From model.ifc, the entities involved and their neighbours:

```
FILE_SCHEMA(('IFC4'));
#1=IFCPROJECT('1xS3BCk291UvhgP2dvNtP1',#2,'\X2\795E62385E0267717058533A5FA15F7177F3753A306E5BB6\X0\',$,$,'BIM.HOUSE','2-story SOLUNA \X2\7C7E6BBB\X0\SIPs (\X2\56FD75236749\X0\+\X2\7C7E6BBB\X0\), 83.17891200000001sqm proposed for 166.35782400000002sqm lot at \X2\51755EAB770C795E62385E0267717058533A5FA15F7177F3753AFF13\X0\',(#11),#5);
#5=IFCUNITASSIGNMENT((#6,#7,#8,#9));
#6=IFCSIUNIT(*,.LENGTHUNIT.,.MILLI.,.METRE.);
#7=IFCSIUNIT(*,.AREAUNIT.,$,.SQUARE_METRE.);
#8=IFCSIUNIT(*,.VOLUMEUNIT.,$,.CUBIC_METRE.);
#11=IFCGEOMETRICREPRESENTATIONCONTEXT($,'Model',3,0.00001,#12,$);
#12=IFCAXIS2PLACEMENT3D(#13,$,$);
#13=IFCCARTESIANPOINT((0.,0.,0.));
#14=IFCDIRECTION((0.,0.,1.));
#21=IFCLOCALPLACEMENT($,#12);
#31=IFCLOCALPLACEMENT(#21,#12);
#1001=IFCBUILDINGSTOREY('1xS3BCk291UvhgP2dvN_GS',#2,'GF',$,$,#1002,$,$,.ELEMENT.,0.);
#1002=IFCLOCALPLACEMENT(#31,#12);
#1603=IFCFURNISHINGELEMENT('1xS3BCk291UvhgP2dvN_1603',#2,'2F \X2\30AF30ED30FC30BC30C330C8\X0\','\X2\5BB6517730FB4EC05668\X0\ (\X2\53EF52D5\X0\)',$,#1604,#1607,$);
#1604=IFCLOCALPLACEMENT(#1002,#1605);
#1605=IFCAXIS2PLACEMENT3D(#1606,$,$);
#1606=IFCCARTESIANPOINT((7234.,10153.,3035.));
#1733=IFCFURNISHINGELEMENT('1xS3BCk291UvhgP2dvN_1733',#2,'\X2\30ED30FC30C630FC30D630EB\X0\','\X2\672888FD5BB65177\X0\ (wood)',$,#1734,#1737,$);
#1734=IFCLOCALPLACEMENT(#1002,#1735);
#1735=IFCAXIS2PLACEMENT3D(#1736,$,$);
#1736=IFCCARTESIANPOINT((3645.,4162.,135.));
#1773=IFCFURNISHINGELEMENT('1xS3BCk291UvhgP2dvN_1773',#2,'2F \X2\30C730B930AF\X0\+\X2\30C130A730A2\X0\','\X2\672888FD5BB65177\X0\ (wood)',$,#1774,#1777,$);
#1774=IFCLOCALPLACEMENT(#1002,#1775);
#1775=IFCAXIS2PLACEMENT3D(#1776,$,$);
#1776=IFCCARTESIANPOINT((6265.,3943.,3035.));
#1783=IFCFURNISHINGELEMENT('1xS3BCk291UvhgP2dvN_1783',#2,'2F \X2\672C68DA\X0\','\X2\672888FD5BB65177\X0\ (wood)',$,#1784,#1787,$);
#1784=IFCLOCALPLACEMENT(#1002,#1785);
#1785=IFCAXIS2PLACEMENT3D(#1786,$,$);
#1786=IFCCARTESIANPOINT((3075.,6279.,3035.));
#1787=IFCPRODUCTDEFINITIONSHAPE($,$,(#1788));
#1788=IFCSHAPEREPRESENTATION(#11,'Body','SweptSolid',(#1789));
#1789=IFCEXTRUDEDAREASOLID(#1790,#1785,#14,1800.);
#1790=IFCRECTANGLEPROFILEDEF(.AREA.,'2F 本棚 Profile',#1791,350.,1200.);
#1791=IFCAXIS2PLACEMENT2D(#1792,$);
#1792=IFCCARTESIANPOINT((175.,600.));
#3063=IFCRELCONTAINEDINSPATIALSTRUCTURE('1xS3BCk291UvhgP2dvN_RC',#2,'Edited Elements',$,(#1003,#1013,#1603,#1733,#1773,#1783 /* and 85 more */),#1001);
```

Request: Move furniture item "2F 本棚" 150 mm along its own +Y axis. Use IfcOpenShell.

```python
import ifcopenshell
import ifcopenshell.api.geometry
import ifcopenshell.util.placement

model = ifcopenshell.open("model.ifc")

item = model.by_guid("1xS3BCk291UvhgP2dvN_1783")
matrix = ifcopenshell.util.placement.get_local_placement(item.ObjectPlacement)
matrix[:3, 3] += matrix[:3, 1] * 150.0
ifcopenshell.api.geometry.edit_object_placement(model, product=item, matrix=matrix, is_si=False)

print(ifcopenshell.util.placement.get_local_placement(item.ObjectPlacement).round(3) + 0.0)

model.write("model_v2.ifc")
```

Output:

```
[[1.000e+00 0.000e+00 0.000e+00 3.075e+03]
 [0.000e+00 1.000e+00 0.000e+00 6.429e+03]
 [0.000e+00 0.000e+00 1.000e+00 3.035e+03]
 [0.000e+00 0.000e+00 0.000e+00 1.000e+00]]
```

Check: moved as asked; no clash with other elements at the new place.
